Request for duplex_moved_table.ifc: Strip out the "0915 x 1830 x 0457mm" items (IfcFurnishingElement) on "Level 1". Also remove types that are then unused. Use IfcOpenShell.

First a look at what the model holds.

```python
import ifcopenshell
import ifcopenshell.util.element

model = ifcopenshell.open("duplex_moved_table.ifc")
print(model.schema)
storey = next(s for s in model.by_type("IfcBuildingStorey") if s.Name == "Level 1")
furniture = [e for e in ifcopenshell.util.element.get_decomposition(storey) if e.is_a("IfcFurnishingElement")]
seen = {}
for e in furniture:
    element_type = ifcopenshell.util.element.get_type(e)
    name = element_type.Name if element_type not in (None, e) else None
    seen[name] = seen.get(name, 0) + 1
for name, count in sorted(seen.items(), key=str):
    print(count, "x", name)
```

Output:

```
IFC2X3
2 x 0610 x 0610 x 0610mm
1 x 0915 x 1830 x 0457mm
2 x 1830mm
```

```python
import ifcopenshell
import ifcopenshell.api.root
import ifcopenshell.util.element

model = ifcopenshell.open("duplex_moved_table.ifc")

storey = next(s for s in model.by_type("IfcBuildingStorey") if s.Name == "Level 1")
furniture = [e for e in ifcopenshell.util.element.get_decomposition(storey) if e.is_a("IfcFurnishingElement")]
targets = [e for e in furniture if (t := ifcopenshell.util.element.get_type(e)) not in (None, e) and t.Name == "0915 x 1830 x 0457mm"]
types = {ifcopenshell.util.element.get_type(e) for e in targets} - {None, *targets}

for e in targets:
    ifcopenshell.api.root.remove_product(model, product=e)
print(len(targets), "removed")

unused = [t for t in types if not ifcopenshell.util.element.get_types(t)]
for t in unused:
    ifcopenshell.api.root.remove_product(model, product=t)
print(len(unused), "unused types removed")

model.write("duplex_moved_table_updated.ifc")
```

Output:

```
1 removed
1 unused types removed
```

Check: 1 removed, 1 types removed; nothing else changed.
